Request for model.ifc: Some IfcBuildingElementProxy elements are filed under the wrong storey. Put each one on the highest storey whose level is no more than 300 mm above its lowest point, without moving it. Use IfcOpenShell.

First a look at what the model holds.

```python
import ifcopenshell
import ifcopenshell.util.element
import ifcopenshell.util.placement

model = ifcopenshell.open("model.ifc")
print(model.schema)
for storey in model.by_type("IfcBuildingStorey"):
    level = ifcopenshell.util.placement.get_storey_elevation(storey)
    count = sum(e.is_a("IfcBuildingElementProxy") for e in ifcopenshell.util.element.get_contained(storey))
    print(storey.id(), storey.Name, round(level, 3), count, sep=" | ")
```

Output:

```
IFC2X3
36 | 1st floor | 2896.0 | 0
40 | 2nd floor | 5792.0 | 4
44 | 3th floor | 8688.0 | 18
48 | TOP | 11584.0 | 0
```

```python
import ifcopenshell
import ifcopenshell.api.spatial
import ifcopenshell.geom
import ifcopenshell.util.element
import ifcopenshell.util.placement
import ifcopenshell.util.shape
import ifcopenshell.util.unit

model = ifcopenshell.open("model.ifc")
unit_scale = ifcopenshell.util.unit.calculate_unit_scale(model)
settings = ifcopenshell.geom.settings()

levels = sorted(
    ((ifcopenshell.util.placement.get_storey_elevation(s) * unit_scale, s) for s in model.by_type("IfcBuildingStorey")),
    key=lambda pair: pair[0],
)

for e in model.by_type("IfcBuildingElementProxy"):
    current = e.ContainedInStructure[0].RelatingStructure if e.ContainedInStructure else None
    if current is None or not current.is_a("IfcBuildingStorey"):
        continue
    shape = ifcopenshell.geom.create_shape(settings, e)
    bottom = ifcopenshell.util.shape.get_shape_bottom_elevation(shape, shape.geometry)
    below = [s for level, s in levels if level <= bottom + 0.3]
    storey = below[-1] if below else levels[0][1]
    if storey != current:
        # assign_container keeps the world position.
        ifcopenshell.api.spatial.assign_container(model, products=[e], relating_structure=storey)
        print(e.id(), current.Name, "->", storey.Name)

model.write("model_updated.ifc")
```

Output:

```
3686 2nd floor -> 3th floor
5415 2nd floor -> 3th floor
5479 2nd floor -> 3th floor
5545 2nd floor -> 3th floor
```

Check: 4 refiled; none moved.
